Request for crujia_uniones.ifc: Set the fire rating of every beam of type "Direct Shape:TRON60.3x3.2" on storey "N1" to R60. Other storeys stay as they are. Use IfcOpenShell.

First a look at what the model holds.

```python
import ifcopenshell
import ifcopenshell.util.element

model = ifcopenshell.open("crujia_uniones.ifc")
print(model.schema)
storey = next(s for s in model.by_type("IfcBuildingStorey") if s.Name == "N1")
beams = [e for e in ifcopenshell.util.element.get_decomposition(storey) if e.is_a("IfcBeam")]
seen = {}
for e in beams:
    element_type = ifcopenshell.util.element.get_type(e)
    key = (element_type.Name if element_type != e and element_type else None, ifcopenshell.util.element.get_pset(e, "Pset_BeamCommon", "FireRating"))
    seen[key] = seen.get(key, 0) + 1
for (name, value), count in sorted(seen.items(), key=str):
    print(count, "x", name, "|", value)
```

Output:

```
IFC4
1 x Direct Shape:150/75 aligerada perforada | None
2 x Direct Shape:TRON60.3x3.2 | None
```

```python
import ifcopenshell
import ifcopenshell.api.pset
import ifcopenshell.util.element

model = ifcopenshell.open("crujia_uniones.ifc")

storey = next(s for s in model.by_type("IfcBuildingStorey") if s.Name == "N1")
beams = [e for e in ifcopenshell.util.element.get_decomposition(storey) if e.is_a("IfcBeam")]

count = 0
for e in beams:
    element_type = ifcopenshell.util.element.get_type(e)
    if element_type in (None, e) or element_type.Name != "Direct Shape:TRON60.3x3.2":
        continue
    # add_pset returns the element's existing set when there is one.
    pset = ifcopenshell.api.pset.add_pset(model, product=e, name="Pset_BeamCommon")
    ifcopenshell.api.pset.edit_pset(model, pset=pset, properties={"FireRating": "R60"})
    count += 1

print(count, "beams updated")

model.write("crujia_uniones_edited.ifc")
```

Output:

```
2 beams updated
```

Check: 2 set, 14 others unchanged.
